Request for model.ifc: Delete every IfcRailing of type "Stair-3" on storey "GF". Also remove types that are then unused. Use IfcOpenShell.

First a look at what the model holds.

```python
import ifcopenshell
import ifcopenshell.util.element

model = ifcopenshell.open("model.ifc")
print(model.schema)
storey = next(s for s in model.by_type("IfcBuildingStorey") if s.Name == "GF")
railings = [e for e in ifcopenshell.util.element.get_decomposition(storey) if e.is_a("IfcRailing")]
seen = {}
for e in railings:
    element_type = ifcopenshell.util.element.get_type(e)
    name = element_type.Name if element_type not in (None, e) else None
    seen[name] = seen.get(name, 0) + 1
for name, count in sorted(seen.items(), key=str):
    print(count, "x", name)
```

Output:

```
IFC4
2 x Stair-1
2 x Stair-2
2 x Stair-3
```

```python
import ifcopenshell
import ifcopenshell.api.root
import ifcopenshell.util.element

model = ifcopenshell.open("model.ifc")

storey = next(s for s in model.by_type("IfcBuildingStorey") if s.Name == "GF")
railings = [e for e in ifcopenshell.util.element.get_decomposition(storey) if e.is_a("IfcRailing")]
targets = [e for e in railings if (t := ifcopenshell.util.element.get_type(e)) not in (None, e) and t.Name == "Stair-3"]
types = {ifcopenshell.util.element.get_type(e) for e in targets} - {None, *targets}

for e in targets:
    ifcopenshell.api.root.remove_product(model, product=e)
print(len(targets), "removed")

unused = [t for t in types if not ifcopenshell.util.element.get_types(t)]
for t in unused:
    ifcopenshell.api.root.remove_product(model, product=t)
print(len(unused), "unused types removed")

model.write("model_edited.ifc")
```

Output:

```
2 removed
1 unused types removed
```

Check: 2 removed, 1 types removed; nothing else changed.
